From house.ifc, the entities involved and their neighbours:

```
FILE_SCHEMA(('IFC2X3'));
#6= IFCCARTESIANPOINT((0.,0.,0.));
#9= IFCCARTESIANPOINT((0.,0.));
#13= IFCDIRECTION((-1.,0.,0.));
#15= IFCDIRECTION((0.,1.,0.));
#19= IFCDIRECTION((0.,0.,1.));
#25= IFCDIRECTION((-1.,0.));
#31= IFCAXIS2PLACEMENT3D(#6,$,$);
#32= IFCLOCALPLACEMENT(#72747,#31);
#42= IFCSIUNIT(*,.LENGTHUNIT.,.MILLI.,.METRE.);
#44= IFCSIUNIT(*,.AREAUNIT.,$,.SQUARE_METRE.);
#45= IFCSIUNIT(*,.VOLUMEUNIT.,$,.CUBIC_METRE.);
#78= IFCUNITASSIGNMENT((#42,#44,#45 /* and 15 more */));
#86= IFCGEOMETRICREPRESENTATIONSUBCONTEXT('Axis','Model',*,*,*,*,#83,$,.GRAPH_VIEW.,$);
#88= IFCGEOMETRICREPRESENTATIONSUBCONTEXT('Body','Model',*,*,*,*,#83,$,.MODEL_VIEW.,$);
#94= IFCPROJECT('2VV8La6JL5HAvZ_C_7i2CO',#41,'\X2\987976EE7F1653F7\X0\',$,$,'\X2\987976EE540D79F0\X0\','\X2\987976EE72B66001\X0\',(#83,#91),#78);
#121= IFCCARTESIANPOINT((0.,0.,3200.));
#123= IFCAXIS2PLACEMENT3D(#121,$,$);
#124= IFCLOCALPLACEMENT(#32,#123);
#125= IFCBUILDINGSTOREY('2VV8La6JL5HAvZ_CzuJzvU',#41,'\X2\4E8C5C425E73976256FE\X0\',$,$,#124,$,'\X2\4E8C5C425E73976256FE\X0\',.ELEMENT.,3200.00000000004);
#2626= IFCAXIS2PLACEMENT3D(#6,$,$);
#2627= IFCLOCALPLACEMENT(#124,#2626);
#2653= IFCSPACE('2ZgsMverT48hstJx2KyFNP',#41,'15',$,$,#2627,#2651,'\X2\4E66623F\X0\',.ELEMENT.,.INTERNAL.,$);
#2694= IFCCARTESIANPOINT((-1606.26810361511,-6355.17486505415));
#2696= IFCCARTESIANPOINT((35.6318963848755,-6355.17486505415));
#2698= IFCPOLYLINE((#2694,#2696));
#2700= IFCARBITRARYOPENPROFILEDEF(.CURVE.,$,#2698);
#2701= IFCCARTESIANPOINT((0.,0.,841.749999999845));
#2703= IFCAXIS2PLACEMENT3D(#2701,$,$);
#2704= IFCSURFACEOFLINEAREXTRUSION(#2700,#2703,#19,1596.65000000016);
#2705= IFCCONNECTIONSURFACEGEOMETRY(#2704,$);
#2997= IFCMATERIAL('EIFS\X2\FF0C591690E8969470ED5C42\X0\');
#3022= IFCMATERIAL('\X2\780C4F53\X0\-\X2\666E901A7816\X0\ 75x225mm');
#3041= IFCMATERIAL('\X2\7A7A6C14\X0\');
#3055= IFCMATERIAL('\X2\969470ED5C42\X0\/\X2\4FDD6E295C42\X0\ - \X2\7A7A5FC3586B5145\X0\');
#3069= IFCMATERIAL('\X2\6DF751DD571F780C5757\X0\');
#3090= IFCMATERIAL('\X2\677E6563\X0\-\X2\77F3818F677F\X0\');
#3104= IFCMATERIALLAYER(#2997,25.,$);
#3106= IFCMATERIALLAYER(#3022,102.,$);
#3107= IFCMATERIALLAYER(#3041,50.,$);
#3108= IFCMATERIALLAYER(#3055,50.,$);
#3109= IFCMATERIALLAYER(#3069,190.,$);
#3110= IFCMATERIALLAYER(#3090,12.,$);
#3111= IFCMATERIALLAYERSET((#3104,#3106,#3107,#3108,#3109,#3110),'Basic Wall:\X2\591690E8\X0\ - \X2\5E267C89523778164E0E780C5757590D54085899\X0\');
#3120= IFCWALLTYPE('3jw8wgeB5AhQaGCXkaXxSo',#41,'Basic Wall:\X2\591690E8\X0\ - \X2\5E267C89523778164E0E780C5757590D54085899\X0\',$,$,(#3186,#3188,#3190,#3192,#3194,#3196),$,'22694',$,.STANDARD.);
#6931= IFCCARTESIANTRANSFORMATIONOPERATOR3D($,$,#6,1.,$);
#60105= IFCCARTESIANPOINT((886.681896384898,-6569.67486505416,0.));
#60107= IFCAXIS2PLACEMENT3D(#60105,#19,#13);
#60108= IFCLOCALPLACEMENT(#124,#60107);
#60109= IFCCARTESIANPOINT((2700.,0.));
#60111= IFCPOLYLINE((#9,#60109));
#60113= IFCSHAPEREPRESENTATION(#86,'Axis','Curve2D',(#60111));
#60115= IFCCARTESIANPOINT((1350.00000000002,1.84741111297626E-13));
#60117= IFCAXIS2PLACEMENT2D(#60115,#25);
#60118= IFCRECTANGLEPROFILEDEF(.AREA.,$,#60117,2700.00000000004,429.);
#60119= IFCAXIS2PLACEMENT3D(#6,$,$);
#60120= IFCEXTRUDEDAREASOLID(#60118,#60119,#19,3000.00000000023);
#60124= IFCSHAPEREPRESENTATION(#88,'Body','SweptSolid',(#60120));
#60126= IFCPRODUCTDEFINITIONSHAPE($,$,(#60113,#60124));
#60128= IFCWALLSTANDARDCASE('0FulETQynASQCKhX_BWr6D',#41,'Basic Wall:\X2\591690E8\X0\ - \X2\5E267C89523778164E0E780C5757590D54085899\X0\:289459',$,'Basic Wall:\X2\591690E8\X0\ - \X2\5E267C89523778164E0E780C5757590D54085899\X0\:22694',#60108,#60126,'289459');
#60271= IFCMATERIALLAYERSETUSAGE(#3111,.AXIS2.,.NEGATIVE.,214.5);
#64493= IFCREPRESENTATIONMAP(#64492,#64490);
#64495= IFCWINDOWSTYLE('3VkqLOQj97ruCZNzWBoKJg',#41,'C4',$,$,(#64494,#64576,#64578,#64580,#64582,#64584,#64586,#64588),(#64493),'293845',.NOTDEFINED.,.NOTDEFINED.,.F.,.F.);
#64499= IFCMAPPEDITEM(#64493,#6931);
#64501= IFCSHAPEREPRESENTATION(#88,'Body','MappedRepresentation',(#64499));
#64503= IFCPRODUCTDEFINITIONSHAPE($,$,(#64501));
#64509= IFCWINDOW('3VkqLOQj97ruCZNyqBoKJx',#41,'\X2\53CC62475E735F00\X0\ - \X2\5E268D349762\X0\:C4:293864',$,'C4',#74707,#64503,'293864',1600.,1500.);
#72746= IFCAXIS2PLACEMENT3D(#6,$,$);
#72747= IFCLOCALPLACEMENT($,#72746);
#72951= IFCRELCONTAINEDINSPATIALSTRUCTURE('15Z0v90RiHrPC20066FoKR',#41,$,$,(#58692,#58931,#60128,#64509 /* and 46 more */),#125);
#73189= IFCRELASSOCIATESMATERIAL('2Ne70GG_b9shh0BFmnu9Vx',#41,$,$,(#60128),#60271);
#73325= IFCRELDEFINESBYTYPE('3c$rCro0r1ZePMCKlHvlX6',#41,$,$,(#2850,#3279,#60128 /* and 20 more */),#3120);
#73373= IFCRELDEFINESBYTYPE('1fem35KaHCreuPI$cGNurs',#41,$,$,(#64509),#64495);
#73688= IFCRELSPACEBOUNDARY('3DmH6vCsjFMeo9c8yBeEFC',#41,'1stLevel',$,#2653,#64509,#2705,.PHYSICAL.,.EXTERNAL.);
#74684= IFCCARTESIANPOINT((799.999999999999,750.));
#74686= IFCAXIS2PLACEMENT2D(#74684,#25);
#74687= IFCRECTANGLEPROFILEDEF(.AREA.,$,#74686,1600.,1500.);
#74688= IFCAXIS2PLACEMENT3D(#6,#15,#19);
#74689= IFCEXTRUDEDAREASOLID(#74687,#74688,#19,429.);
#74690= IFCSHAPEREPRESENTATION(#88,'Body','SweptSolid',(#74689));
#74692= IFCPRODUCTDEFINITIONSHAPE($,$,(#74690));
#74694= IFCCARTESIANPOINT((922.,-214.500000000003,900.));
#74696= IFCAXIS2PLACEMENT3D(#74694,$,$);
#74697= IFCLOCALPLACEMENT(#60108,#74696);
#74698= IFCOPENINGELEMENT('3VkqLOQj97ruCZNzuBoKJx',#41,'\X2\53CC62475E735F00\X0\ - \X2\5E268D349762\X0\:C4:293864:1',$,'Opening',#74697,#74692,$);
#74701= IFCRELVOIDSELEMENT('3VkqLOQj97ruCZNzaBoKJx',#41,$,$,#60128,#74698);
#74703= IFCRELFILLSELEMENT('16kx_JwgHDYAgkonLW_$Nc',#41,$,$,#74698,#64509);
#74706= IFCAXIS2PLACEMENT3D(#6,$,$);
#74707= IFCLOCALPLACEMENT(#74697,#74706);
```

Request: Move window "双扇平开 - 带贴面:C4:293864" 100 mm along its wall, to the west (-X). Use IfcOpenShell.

```python
import numpy as np
import ifcopenshell
import ifcopenshell.api.geometry
import ifcopenshell.util.placement
import ifcopenshell.util.unit

model = ifcopenshell.open("house.ifc")
unit_scale = ifcopenshell.util.unit.calculate_unit_scale(model)

window = model.by_guid("3VkqLOQj97ruCZNyqBoKJx")
opening = window.FillsVoids[0].RelatingOpeningElement
wall = opening.VoidsElements[0].RelatingBuildingElement

wall_matrix = ifcopenshell.util.placement.get_local_placement(wall.ObjectPlacement)
shift = wall_matrix[:3, 0] * 0.1 / unit_scale
before = ifcopenshell.util.placement.get_local_placement(window.ObjectPlacement)[:3, 3].copy()

# The window is placed relative to its opening, so it follows when the opening moves.
matrix = ifcopenshell.util.placement.get_local_placement(opening.ObjectPlacement)
matrix[:3, 3] += shift
ifcopenshell.api.geometry.edit_object_placement(
    model, product=opening, matrix=matrix, is_si=False, should_transform_children=True
)

# Space boundary surfaces are stored in each space's coordinates; move them too.
for rel in window.ProvidesBoundaries:
    if not rel.ConnectionGeometry:
        continue
    surface = rel.ConnectionGeometry.SurfaceOnRelatingElement
    space_matrix = ifcopenshell.util.placement.get_local_placement(rel.RelatingSpace.ObjectPlacement)
    point = np.array(surface.Position.Location.Coordinates) + space_matrix[:3, :3].T @ shift
    surface.Position = model.createIfcAxis2Placement3D(
        model.createIfcCartesianPoint(point.tolist()), surface.Position.Axis, surface.Position.RefDirection
    )

after = ifcopenshell.util.placement.get_local_placement(window.ObjectPlacement)[:3, 3]
print("window moved by", (after - before).round(3) + 0.0)

model.write("house-out.ifc")
```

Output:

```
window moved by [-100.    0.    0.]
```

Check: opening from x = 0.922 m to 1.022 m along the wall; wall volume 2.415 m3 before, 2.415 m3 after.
